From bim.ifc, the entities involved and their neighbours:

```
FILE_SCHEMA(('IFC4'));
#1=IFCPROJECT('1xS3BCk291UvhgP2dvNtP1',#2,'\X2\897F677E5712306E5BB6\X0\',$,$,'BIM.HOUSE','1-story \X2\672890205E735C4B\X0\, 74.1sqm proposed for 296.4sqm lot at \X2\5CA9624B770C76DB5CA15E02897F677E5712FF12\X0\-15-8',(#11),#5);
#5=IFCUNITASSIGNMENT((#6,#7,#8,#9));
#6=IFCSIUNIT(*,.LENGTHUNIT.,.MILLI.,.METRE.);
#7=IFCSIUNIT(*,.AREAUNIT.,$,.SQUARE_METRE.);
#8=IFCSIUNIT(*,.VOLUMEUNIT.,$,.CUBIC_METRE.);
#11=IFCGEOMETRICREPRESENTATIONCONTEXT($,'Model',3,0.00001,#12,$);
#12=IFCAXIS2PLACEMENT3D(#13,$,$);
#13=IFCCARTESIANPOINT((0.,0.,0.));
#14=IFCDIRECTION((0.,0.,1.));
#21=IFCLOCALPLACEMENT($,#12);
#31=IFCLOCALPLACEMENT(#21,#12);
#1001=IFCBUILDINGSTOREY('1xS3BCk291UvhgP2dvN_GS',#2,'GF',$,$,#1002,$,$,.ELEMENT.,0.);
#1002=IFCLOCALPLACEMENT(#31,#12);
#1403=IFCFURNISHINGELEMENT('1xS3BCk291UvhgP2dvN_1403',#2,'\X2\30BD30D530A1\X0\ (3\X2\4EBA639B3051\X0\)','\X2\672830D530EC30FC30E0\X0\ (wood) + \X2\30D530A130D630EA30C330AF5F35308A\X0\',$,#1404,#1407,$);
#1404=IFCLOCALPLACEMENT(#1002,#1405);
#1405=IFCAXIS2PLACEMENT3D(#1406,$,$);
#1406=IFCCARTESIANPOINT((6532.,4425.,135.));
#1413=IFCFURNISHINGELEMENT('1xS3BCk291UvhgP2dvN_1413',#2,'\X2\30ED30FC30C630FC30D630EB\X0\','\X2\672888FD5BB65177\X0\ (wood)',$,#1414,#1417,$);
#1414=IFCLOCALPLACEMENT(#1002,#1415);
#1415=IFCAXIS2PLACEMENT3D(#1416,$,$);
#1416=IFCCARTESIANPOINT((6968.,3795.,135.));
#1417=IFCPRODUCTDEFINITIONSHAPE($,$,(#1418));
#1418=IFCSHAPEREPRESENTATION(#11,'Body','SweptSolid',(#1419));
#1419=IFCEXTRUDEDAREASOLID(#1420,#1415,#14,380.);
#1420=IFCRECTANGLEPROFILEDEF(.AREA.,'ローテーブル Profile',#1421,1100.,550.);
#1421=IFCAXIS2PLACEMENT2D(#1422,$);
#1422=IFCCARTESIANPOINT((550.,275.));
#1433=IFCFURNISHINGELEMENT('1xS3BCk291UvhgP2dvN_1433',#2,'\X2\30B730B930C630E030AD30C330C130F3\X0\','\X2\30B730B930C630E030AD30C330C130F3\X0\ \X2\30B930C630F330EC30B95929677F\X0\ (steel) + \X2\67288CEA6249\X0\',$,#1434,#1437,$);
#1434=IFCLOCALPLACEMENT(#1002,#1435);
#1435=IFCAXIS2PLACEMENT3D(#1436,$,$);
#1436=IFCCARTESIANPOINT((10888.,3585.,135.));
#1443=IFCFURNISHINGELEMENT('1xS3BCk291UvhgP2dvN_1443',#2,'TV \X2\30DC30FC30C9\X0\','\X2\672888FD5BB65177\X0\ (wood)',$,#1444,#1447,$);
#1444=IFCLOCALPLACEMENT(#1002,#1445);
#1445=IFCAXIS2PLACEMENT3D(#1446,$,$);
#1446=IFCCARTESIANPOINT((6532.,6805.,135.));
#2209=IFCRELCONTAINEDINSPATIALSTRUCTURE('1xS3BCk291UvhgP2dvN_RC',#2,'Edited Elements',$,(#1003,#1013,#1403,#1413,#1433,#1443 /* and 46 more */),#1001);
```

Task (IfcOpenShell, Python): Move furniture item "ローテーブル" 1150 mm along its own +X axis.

```python
import ifcopenshell
import ifcopenshell.api.geometry
import ifcopenshell.util.placement
import ifcopenshell.util.unit

model = ifcopenshell.open("bim.ifc")
unit_scale = ifcopenshell.util.unit.calculate_unit_scale(model)

item = model.by_id(1413)
matrix = ifcopenshell.util.placement.get_local_placement(item.ObjectPlacement)
matrix[:3, 3] += matrix[:3, 0] * 1.15 / unit_scale
ifcopenshell.api.geometry.edit_object_placement(model, product=item, matrix=matrix, is_si=False)

print(ifcopenshell.util.placement.get_local_placement(item.ObjectPlacement).round(3) + 0.0)

model.write("bim_edited.ifc")
```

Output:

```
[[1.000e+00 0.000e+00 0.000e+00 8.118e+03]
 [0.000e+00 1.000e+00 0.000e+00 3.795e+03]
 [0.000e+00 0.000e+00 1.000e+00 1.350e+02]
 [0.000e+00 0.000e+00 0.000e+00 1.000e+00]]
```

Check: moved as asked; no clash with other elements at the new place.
